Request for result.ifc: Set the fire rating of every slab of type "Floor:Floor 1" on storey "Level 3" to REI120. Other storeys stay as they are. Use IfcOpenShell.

First a look at what the model holds.

```python
import ifcopenshell
import ifcopenshell.util.element

model = ifcopenshell.open("result.ifc")
print(model.schema)
storey = next(s for s in model.by_type("IfcBuildingStorey") if s.Name == "Level 3")
slabs = [e for e in ifcopenshell.util.element.get_decomposition(storey) if e.is_a("IfcSlab")]
seen = {}
for e in slabs:
    element_type = ifcopenshell.util.element.get_type(e)
    key = (element_type.Name if element_type != e and element_type else None, ifcopenshell.util.element.get_pset(e, "Pset_SlabCommon", "FireRating"))
    seen[key] = seen.get(key, 0) + 1
for (name, value), count in sorted(seen.items(), key=str):
    print(count, "x", name, "|", value)
```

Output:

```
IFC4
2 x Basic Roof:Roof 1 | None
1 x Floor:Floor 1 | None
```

```python
import ifcopenshell
import ifcopenshell.api.pset
import ifcopenshell.util.element

model = ifcopenshell.open("result.ifc")

storey = next(s for s in model.by_type("IfcBuildingStorey") if s.Name == "Level 3")
slabs = [e for e in ifcopenshell.util.element.get_decomposition(storey) if e.is_a("IfcSlab")]

count = 0
for e in slabs:
    element_type = ifcopenshell.util.element.get_type(e)
    if element_type in (None, e) or element_type.Name != "Floor:Floor 1":
        continue
    # add_pset returns the element's existing set when there is one.
    pset = ifcopenshell.api.pset.add_pset(model, product=e, name="Pset_SlabCommon")
    ifcopenshell.api.pset.edit_pset(model, pset=pset, properties={"FireRating": "REI120"})
    count += 1

print(count, "slabs updated")

model.write("result_v2.ifc")
```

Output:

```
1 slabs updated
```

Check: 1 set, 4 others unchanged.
